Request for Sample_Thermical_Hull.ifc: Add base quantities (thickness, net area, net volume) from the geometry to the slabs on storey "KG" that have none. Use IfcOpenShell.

First a look at what the model holds.

```python
import ifcopenshell
import ifcopenshell.util.element
import ifcopenshell.util.unit

model = ifcopenshell.open("Sample_Thermical_Hull.ifc")
print(model.schema)
for unit_type in ("LENGTHUNIT", "AREAUNIT", "VOLUMEUNIT"):
    print(unit_type, ifcopenshell.util.unit.calculate_unit_scale(model, unit_type))
storey = next(s for s in model.by_type("IfcBuildingStorey") if s.Name == "KG")
slabs = [e for e in ifcopenshell.util.element.get_decomposition(storey) if e.is_a("IfcSlab")]
for e in sorted(slabs, key=lambda e: e.id()):
    print(e.id(), e.is_a(), e.Name, list(ifcopenshell.util.element.get_psets(e, qtos_only=True)), sep=" | ")
```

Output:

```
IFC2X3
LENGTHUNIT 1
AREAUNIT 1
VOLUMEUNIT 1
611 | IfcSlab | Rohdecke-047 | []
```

```python
import ifcopenshell
import ifcopenshell.api.pset
import ifcopenshell.geom
import ifcopenshell.util.element
import ifcopenshell.util.shape
import ifcopenshell.util.unit

model = ifcopenshell.open("Sample_Thermical_Hull.ifc")
unit_scale = ifcopenshell.util.unit.calculate_unit_scale(model)
area_scale = ifcopenshell.util.unit.calculate_unit_scale(model, "AREAUNIT")
volume_scale = ifcopenshell.util.unit.calculate_unit_scale(model, "VOLUMEUNIT")
settings = ifcopenshell.geom.settings()

storey = next(s for s in model.by_type("IfcBuildingStorey") if s.Name == "KG")
slabs = [e for e in ifcopenshell.util.element.get_decomposition(storey) if e.is_a("IfcSlab")]

for e in sorted(slabs, key=lambda e: e.id()):
    if ifcopenshell.util.element.get_psets(e, qtos_only=True, should_inherit=False):
        continue
    # Geometry comes back in metres, in the element's own axes.
    shape = ifcopenshell.geom.create_shape(settings, e)
    values = {
        "Width": ifcopenshell.util.shape.get_z(shape.geometry) / unit_scale,
        "NetArea": ifcopenshell.util.shape.get_footprint_area(shape.geometry) / area_scale,
        "NetVolume": ifcopenshell.util.shape.get_volume(shape.geometry) / volume_scale,
    }
    qto = ifcopenshell.api.pset.add_qto(model, product=e, name="BaseQuantities")
    ifcopenshell.api.pset.edit_qto(model, qto=qto, properties=values)
    print(e.id(), {k: round(v, 3) for k, v in values.items()})

model.write("Sample_Thermical_Hull_v2.ifc")
```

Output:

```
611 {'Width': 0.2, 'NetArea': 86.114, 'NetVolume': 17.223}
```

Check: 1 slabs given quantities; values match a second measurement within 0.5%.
